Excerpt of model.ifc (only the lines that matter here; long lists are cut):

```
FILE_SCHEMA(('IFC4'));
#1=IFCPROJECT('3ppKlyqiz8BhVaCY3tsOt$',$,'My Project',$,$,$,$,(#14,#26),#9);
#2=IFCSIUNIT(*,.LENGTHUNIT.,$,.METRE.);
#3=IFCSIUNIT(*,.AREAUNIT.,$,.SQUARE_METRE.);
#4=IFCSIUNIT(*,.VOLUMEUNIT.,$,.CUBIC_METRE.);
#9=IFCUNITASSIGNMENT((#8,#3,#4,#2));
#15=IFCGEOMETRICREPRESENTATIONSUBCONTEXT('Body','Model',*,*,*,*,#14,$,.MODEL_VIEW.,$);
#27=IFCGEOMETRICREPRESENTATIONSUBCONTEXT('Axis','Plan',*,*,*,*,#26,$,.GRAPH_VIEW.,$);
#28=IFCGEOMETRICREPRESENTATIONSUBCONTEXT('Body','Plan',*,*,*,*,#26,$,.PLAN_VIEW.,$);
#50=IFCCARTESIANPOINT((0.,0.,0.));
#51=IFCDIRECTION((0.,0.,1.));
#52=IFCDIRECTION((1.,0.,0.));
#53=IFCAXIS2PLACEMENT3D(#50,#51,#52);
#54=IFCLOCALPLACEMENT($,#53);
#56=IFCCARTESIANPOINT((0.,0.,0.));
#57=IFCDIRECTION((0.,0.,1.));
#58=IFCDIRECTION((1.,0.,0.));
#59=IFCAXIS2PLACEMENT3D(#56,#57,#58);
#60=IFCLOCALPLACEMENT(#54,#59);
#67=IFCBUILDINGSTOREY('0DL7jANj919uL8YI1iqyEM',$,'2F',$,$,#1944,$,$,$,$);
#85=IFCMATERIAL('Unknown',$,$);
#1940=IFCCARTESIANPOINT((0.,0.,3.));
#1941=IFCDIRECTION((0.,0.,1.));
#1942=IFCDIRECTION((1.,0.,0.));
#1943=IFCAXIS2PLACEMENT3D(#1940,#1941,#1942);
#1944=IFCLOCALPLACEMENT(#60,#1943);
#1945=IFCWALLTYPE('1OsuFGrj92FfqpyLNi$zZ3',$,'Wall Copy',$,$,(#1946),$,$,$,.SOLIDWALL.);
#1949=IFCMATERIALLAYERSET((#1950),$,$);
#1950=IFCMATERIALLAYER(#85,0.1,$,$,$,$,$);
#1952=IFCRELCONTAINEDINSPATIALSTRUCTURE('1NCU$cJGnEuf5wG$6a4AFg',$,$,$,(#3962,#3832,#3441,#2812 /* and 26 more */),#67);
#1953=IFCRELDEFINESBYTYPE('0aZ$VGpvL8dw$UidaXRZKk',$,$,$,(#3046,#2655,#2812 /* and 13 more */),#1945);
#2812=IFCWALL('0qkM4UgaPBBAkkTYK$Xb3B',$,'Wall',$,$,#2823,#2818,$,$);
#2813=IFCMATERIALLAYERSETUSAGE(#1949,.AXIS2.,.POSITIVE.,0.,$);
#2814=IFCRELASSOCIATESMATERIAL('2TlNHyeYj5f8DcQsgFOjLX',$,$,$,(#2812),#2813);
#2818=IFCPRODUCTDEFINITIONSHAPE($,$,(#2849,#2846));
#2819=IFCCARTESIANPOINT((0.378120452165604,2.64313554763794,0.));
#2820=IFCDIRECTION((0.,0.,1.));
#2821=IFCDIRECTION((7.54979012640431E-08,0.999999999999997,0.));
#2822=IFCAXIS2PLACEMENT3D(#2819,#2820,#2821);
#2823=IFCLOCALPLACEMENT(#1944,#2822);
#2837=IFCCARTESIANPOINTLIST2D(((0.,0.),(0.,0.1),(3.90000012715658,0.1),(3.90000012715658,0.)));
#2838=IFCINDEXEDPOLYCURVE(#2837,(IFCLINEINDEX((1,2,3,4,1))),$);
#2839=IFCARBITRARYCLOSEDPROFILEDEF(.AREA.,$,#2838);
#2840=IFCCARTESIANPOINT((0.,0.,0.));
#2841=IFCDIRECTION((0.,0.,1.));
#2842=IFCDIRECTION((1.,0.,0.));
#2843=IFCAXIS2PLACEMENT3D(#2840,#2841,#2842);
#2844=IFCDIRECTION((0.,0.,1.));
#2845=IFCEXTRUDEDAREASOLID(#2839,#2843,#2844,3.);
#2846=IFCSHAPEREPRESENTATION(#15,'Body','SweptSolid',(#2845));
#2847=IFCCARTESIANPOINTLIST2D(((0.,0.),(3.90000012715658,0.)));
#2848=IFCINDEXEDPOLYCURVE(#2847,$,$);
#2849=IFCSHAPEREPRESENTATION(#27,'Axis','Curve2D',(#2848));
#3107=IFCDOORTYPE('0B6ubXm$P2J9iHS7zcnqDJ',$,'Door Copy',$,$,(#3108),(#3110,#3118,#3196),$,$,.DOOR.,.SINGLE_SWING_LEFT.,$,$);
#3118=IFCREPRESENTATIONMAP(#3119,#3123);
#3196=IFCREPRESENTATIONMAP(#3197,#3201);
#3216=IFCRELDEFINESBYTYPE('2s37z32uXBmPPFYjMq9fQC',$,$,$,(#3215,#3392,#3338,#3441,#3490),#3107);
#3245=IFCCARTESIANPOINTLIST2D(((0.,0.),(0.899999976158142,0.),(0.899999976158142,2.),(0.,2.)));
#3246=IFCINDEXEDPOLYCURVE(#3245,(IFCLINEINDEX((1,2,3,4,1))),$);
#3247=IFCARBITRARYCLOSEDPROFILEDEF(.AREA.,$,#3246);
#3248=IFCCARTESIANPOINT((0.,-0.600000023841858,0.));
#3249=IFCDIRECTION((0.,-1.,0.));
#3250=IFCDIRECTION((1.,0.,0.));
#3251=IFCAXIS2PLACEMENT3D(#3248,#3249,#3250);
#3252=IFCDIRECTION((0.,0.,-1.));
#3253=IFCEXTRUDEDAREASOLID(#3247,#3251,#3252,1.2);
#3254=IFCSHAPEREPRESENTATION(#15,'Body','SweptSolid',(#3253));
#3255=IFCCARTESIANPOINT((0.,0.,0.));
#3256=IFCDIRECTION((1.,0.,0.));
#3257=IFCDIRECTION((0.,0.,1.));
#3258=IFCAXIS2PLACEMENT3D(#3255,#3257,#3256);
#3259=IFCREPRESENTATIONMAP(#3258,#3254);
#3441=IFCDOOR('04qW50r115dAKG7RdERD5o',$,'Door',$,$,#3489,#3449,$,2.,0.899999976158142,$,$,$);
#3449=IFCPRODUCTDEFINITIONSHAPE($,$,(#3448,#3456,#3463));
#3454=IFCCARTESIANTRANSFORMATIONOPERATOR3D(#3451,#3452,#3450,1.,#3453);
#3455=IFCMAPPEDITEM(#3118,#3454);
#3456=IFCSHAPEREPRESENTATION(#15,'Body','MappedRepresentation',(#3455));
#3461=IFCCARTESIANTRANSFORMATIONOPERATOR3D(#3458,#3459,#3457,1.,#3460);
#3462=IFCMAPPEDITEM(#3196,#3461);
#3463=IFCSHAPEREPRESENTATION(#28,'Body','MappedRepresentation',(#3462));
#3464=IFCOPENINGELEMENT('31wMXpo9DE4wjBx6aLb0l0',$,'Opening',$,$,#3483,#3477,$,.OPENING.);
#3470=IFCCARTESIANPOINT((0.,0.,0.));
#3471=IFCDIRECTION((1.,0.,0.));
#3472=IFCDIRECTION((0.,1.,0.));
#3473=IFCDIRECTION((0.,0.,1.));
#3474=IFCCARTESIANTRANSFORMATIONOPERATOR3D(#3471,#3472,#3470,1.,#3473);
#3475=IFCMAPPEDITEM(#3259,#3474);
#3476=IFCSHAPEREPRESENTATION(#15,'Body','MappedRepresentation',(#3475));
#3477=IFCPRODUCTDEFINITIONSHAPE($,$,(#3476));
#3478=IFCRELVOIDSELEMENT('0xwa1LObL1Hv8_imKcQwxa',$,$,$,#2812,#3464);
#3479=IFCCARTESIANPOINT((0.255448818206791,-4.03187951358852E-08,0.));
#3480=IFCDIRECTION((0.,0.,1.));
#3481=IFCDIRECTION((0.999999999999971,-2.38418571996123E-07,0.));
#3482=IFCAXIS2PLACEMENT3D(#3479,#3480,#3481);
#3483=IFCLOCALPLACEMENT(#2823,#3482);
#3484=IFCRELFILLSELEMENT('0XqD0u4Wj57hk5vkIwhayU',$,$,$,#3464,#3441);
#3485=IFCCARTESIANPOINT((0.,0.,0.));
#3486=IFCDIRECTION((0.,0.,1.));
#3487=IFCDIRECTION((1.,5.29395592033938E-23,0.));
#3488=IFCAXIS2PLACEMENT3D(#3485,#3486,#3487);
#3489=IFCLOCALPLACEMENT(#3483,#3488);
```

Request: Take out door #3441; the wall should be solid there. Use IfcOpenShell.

```python
import ifcopenshell
import ifcopenshell.api.feature
import ifcopenshell.api.root
import ifcopenshell.geom
import ifcopenshell.util.shape

model = ifcopenshell.open("model.ifc")
settings = ifcopenshell.geom.settings()


def volume(element):
    """Net volume in cubic metres, openings subtracted."""
    shape = ifcopenshell.geom.create_shape(settings, element)
    return ifcopenshell.util.shape.get_volume(shape.geometry)


door = model.by_id(3441)
opening = door.FillsVoids[0].RelatingOpeningElement
wall = opening.VoidsElements[0].RelatingBuildingElement
before = volume(wall)

ifcopenshell.api.root.remove_product(model, product=door)
ifcopenshell.api.feature.remove_feature(model, feature=opening)

after = volume(wall)

print(f"wall volume {before:.3f} -> {after:.3f} m3")

model.write("model_rev.ifc")
```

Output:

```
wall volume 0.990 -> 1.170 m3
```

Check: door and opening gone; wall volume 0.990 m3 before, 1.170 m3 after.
